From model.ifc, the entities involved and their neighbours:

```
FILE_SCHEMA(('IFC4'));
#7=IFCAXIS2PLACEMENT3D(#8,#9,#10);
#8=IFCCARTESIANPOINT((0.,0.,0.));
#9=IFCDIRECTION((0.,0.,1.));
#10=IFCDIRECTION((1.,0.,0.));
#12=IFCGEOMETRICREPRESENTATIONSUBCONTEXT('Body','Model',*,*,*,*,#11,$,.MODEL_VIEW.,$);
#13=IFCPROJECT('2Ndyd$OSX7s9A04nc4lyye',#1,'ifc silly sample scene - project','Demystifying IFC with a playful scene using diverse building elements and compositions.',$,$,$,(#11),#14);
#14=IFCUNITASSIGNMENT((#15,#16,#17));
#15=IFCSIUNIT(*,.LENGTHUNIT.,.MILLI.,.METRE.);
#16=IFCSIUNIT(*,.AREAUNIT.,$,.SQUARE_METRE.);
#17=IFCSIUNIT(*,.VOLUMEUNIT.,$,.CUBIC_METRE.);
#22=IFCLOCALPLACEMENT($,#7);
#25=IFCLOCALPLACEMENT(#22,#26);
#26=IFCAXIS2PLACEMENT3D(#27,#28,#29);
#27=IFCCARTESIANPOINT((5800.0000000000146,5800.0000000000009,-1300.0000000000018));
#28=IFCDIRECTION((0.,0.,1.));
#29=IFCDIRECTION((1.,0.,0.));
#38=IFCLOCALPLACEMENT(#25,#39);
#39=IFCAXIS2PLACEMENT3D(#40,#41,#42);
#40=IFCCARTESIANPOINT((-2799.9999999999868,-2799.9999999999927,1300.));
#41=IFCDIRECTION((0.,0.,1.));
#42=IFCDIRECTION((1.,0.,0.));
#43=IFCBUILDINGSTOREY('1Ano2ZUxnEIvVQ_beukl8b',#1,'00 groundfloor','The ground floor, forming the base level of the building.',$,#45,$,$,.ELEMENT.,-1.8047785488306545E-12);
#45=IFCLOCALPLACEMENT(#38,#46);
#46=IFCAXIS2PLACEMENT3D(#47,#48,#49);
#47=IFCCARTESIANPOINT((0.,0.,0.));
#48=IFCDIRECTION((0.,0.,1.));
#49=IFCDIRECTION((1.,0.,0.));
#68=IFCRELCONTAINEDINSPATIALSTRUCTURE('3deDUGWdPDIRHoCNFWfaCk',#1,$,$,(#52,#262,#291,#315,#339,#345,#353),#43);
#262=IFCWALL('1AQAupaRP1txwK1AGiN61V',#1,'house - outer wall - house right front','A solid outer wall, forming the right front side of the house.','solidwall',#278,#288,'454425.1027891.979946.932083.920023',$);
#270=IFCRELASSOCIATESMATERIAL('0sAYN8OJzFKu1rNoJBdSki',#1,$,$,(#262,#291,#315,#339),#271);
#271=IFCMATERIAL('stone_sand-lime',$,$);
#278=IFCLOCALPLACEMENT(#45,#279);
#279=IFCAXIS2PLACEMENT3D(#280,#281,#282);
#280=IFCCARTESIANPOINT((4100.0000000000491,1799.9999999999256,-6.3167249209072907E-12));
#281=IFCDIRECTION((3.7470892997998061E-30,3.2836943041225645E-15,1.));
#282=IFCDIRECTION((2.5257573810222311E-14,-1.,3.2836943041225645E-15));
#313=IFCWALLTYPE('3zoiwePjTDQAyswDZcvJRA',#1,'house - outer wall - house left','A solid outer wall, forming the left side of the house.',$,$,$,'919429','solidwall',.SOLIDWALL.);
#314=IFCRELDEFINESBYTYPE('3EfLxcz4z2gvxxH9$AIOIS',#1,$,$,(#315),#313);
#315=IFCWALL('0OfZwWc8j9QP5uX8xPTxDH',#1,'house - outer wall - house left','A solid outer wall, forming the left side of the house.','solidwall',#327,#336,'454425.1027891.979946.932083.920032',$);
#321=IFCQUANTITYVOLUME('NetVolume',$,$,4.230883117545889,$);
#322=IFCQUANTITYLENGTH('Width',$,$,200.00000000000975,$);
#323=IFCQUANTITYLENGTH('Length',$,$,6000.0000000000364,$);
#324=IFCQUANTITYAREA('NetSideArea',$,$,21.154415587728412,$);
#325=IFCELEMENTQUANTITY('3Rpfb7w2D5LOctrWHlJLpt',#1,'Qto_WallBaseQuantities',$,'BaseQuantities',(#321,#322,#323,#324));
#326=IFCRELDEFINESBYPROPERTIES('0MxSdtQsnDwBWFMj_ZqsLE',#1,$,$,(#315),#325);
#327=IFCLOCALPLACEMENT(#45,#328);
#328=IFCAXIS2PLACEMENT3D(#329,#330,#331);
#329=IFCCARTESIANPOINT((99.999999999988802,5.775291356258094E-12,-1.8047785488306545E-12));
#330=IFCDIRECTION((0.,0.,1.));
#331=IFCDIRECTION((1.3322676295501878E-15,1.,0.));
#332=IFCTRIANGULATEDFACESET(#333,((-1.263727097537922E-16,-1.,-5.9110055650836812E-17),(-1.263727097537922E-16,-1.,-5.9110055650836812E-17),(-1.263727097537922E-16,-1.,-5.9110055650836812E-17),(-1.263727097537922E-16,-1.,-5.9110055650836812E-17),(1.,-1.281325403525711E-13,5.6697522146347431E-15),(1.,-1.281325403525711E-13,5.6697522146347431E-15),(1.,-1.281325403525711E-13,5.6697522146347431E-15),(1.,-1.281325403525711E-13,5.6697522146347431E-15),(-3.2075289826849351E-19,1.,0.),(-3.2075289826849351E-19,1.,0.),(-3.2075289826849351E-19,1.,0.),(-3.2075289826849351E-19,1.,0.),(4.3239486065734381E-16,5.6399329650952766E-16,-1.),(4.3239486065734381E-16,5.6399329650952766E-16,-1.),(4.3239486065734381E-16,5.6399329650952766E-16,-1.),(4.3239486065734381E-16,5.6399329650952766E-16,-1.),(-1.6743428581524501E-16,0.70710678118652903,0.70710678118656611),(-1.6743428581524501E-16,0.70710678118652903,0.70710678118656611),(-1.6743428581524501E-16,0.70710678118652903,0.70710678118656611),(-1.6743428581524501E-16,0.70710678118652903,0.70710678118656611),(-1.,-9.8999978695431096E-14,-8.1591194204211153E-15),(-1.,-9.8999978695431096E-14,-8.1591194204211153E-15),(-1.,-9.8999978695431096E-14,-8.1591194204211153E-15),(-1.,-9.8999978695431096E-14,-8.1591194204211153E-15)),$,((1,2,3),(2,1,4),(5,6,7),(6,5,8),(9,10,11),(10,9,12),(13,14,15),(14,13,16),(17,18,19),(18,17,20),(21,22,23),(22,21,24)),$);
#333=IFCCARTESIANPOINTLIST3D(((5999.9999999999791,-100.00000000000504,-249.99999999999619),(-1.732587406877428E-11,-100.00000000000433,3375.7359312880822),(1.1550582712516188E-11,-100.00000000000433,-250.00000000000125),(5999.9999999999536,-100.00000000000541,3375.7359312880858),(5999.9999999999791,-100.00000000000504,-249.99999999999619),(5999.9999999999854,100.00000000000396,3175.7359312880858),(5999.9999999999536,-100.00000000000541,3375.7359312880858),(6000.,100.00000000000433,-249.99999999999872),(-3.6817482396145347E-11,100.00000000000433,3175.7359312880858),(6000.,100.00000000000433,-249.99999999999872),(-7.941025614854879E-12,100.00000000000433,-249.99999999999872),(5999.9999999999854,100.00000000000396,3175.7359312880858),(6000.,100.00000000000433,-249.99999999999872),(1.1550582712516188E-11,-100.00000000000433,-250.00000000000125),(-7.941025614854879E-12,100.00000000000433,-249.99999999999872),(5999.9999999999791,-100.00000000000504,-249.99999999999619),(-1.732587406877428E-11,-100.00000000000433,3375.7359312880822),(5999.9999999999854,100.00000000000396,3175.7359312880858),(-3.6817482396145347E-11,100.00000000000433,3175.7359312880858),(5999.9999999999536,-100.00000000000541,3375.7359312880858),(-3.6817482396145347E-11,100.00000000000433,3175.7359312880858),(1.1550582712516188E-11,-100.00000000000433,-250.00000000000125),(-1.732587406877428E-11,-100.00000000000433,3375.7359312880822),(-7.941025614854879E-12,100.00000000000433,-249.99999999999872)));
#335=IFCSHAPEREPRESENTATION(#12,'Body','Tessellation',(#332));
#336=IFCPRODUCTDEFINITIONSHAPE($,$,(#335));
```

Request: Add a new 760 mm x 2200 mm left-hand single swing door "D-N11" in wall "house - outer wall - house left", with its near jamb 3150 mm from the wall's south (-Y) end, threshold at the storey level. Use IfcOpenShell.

```python
import numpy as np
import ifcopenshell
import ifcopenshell.api.feature
import ifcopenshell.api.geometry
import ifcopenshell.api.pset
import ifcopenshell.api.root
import ifcopenshell.api.spatial
import ifcopenshell.geom
import ifcopenshell.util.element
import ifcopenshell.util.placement
import ifcopenshell.util.representation
import ifcopenshell.util.shape
import ifcopenshell.util.unit

model = ifcopenshell.open("model.ifc")
unit_scale = ifcopenshell.util.unit.calculate_unit_scale(model)
area_scale = ifcopenshell.util.unit.calculate_unit_scale(model, "AREAUNIT")
volume_scale = ifcopenshell.util.unit.calculate_unit_scale(model, "VOLUMEUNIT")
settings = ifcopenshell.geom.settings()


def volume(element):
    """Net volume in cubic metres, openings subtracted."""
    shape = ifcopenshell.geom.create_shape(settings, element)
    return ifcopenshell.util.shape.get_volume(shape.geometry)


wall = model.by_guid("0OfZwWc8j9QP5uX8xPTxDH")
storey = ifcopenshell.util.element.get_container(wall, ifc_class="IfcBuildingStorey")
context = ifcopenshell.util.representation.get_context(model, "Model", "Body", "MODEL_VIEW")
before = volume(wall)

width, height, from_end, sill = 0.76, 2.2, 3.15, 0.0  # metres

# The wall runs along its own X axis, and the end named is its -X end.
wall_shape = ifcopenshell.geom.create_shape(settings, wall)
x, y, z = ifcopenshell.util.shape.get_vertices(wall_shape.geometry).T
start = x.min() + from_end
face, thickness = float(y.min()), float(y.max() - y.min())
wall_matrix = ifcopenshell.util.placement.get_local_placement(wall.ObjectPlacement)
level = ifcopenshell.util.placement.get_local_placement(storey.ObjectPlacement)[2, 3]


def in_wall(x, y):
    """Placement at x, y metres in the wall's axes, at sill height."""
    matrix = wall_matrix.copy()
    matrix[:, 3] = wall_matrix @ np.array([x / unit_scale, y / unit_scale, 0.0, 1.0])
    matrix[2, 3] = level + sill / unit_scale
    return matrix


# Opening: a box that overshoots both wall faces by 50 mm.
opening = ifcopenshell.api.root.create_entity(model, ifc_class="IfcOpeningElement", predefined_type="OPENING")
box = ifcopenshell.api.geometry.add_wall_representation(
    model, context=context, length=width, height=height, thickness=thickness + 0.1
)
ifcopenshell.api.geometry.assign_representation(model, product=opening, representation=box)
ifcopenshell.api.geometry.edit_object_placement(model, product=opening, matrix=in_wall(start, face - 0.05), is_si=False)
ifcopenshell.api.feature.add_feature(model, feature=opening, element=wall)

door = ifcopenshell.api.root.create_entity(model, ifc_class="IfcDoor", name="D-N11", predefined_type="DOOR")
door.OverallWidth, door.OverallHeight = width / unit_scale, height / unit_scale
door.OperationType = "SINGLE_SWING_LEFT"
body = ifcopenshell.api.geometry.add_door_representation(
    model,
    context=context,
    overall_width=door.OverallWidth,
    overall_height=door.OverallHeight,
    operation_type="SINGLE_SWING_LEFT",
    lining_properties={"LiningDepth": thickness / unit_scale, "ThresholdDepth": thickness / unit_scale},
)
ifcopenshell.api.geometry.assign_representation(model, product=door, representation=body)
ifcopenshell.api.spatial.assign_container(model, products=[door], relating_structure=storey)
ifcopenshell.api.feature.add_filling(model, opening=opening, element=door)

# The lining spans the wall, so the door starts at the wall face.
ifcopenshell.api.geometry.edit_object_placement(model, product=door, matrix=in_wall(start, face), is_si=False)

after = volume(wall)

# Update the wall's stored quantities.
qto = model.by_id(ifcopenshell.util.element.get_pset(wall, "Qto_WallBaseQuantities", should_inherit=False)["id"])
ifcopenshell.api.pset.edit_qto(model, qto=qto, properties={
    "NetVolume": after / volume_scale,
    "NetSideArea": after / thickness / area_scale,
})

print(f"wall volume {before:.3f} -> {after:.3f} m3")

model.write("model_updated.ifc")
```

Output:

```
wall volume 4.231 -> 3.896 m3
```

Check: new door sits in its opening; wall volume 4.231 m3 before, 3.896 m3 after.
